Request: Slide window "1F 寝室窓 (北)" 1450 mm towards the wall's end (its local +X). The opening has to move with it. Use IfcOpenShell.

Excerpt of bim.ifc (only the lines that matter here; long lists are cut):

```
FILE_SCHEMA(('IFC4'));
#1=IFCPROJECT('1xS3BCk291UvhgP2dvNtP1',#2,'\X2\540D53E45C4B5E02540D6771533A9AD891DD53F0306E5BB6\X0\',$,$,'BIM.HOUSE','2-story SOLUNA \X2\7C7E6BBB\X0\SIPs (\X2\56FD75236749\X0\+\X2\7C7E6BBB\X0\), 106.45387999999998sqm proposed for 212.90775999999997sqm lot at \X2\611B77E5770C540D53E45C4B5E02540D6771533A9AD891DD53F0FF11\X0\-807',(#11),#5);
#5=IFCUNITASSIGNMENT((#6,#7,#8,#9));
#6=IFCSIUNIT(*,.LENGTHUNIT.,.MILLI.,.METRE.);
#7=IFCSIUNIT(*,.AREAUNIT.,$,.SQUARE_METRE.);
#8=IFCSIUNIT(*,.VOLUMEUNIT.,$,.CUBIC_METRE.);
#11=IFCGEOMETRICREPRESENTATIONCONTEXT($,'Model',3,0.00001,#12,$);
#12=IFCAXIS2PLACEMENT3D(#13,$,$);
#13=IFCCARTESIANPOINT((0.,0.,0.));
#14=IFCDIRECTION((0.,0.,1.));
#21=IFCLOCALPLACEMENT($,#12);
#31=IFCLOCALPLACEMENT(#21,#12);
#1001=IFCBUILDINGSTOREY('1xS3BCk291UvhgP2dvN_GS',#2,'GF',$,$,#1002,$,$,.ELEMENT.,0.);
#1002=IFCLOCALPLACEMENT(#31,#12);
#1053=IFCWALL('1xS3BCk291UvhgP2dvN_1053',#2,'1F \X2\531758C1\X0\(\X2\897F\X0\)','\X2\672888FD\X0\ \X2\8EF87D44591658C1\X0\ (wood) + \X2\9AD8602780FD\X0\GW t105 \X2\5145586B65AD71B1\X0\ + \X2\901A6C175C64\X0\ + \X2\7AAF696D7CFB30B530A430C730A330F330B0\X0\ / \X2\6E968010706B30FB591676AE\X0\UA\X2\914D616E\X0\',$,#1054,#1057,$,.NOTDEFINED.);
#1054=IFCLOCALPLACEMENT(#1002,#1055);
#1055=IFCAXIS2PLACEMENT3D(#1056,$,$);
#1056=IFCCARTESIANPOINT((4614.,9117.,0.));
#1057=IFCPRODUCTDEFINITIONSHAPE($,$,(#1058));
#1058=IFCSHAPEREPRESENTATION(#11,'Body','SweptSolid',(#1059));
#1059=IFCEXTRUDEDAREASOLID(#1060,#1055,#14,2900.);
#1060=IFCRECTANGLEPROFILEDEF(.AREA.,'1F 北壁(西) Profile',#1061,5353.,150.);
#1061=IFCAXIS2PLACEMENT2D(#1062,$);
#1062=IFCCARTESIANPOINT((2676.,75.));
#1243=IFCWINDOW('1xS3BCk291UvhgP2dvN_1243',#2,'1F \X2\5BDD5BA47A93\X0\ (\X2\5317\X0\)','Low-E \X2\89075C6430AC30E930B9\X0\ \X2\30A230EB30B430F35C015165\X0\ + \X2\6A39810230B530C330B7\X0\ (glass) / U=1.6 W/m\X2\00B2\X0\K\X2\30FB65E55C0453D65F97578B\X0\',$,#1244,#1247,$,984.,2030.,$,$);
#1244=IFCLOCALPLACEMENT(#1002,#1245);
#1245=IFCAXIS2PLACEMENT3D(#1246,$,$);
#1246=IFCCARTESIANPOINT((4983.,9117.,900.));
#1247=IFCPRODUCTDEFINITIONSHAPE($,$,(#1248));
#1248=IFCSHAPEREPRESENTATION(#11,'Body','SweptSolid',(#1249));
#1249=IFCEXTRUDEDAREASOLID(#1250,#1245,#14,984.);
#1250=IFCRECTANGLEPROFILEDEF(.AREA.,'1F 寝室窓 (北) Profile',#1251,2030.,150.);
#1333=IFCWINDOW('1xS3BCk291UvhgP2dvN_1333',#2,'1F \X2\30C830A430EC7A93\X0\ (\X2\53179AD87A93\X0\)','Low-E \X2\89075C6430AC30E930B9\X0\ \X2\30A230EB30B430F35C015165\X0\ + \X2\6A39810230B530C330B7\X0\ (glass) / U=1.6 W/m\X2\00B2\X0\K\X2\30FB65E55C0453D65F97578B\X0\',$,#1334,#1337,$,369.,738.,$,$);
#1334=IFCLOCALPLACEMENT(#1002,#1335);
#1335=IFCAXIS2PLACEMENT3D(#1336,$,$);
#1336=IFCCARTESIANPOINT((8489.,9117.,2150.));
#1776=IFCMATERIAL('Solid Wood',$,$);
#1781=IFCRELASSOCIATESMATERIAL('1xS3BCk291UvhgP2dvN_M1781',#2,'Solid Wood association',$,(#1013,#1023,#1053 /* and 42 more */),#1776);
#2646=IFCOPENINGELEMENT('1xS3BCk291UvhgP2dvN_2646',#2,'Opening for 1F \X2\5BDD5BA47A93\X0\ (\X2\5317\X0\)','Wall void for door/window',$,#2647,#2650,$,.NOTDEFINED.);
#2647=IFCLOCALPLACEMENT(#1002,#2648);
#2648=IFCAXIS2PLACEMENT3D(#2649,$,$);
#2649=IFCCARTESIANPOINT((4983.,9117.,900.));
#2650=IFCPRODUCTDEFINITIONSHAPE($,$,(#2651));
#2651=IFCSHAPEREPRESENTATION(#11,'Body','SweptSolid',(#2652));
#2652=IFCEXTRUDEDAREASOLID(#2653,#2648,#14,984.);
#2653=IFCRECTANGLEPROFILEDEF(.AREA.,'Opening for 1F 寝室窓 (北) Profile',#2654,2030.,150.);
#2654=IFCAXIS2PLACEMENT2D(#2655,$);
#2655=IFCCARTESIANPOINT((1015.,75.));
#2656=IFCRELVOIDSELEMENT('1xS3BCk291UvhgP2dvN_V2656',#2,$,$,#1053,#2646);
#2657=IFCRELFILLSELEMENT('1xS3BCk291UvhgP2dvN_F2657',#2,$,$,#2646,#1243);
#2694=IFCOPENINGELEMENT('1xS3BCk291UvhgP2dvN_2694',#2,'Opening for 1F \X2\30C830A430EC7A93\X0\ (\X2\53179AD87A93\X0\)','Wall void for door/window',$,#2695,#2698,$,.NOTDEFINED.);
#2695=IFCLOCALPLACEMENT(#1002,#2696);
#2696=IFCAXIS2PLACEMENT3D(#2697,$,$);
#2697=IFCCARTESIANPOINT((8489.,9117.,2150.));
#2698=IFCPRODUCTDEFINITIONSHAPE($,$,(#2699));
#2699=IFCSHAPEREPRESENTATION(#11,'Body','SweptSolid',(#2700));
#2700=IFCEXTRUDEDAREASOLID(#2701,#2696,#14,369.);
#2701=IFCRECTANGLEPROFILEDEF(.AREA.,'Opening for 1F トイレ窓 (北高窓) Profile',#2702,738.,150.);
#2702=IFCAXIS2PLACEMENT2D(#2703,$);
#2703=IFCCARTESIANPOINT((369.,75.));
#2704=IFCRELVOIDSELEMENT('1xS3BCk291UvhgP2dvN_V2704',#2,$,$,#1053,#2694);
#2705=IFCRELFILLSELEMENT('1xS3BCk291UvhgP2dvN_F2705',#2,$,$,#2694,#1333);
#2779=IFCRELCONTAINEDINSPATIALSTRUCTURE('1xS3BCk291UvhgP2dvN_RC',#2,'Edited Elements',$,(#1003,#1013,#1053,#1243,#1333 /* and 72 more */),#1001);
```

```python
import ifcopenshell
import ifcopenshell.api.geometry
import ifcopenshell.util.placement

model = ifcopenshell.open("bim.ifc")

window = model.by_id(1243)
opening = window.FillsVoids[0].RelatingOpeningElement
wall = opening.VoidsElements[0].RelatingBuildingElement

wall_matrix = ifcopenshell.util.placement.get_local_placement(wall.ObjectPlacement)
shift = wall_matrix[:3, 0] * 1450.0
before = ifcopenshell.util.placement.get_local_placement(window.ObjectPlacement)[:3, 3].copy()

# The window is not placed relative to its opening, so move both.
for product in (opening, window):
    matrix = ifcopenshell.util.placement.get_local_placement(product.ObjectPlacement)
    matrix[:3, 3] += shift
    ifcopenshell.api.geometry.edit_object_placement(model, product=product, matrix=matrix, is_si=False)

after = ifcopenshell.util.placement.get_local_placement(window.ObjectPlacement)[:3, 3]
print("window moved by", (after - before).round(3) + 0.0)

model.write("bim_rev.ifc")
```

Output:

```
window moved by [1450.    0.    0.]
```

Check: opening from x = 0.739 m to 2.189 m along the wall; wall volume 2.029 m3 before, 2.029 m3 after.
